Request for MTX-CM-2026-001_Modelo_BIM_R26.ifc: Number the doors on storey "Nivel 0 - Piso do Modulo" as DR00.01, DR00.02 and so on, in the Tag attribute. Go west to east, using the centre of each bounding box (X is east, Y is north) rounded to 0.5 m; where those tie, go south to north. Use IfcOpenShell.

First a look at what the model holds.

```python
import ifcopenshell
import ifcopenshell.util.element
import ifcopenshell.util.placement

model = ifcopenshell.open("MTX-CM-2026-001_Modelo_BIM_R26.ifc")
print(model.schema)
storey = next(s for s in model.by_type("IfcBuildingStorey") if s.Name == "Nivel 0 - Piso do Modulo")
doors = [e for e in ifcopenshell.util.element.get_decomposition(storey) if e.is_a("IfcDoor")]
for e in sorted(doors, key=lambda e: e.id()):
    origin = ifcopenshell.util.placement.get_local_placement(e.ObjectPlacement)[:3, 3]
    print(e.id(), e.Tag, e.Name, origin.round(2) + 0.0, sep=" | ")
```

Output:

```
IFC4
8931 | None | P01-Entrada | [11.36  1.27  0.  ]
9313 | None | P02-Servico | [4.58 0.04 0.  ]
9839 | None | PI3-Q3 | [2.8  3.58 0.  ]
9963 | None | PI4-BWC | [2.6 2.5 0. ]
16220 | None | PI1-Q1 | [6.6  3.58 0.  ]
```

```python
import ifcopenshell
import ifcopenshell.geom
import ifcopenshell.util.element
import ifcopenshell.util.shape

model = ifcopenshell.open("MTX-CM-2026-001_Modelo_BIM_R26.ifc")
settings = ifcopenshell.geom.settings()
settings.set("use-world-coords", True)


def centre(element):
    shape = ifcopenshell.geom.create_shape(settings, element)
    return ifcopenshell.util.shape.get_bbox_centroid(shape.geometry)


storey = next(s for s in model.by_type("IfcBuildingStorey") if s.Name == "Nivel 0 - Piso do Modulo")
doors = [e for e in ifcopenshell.util.element.get_decomposition(storey) if e.is_a("IfcDoor")]

# Insertion points can sit at a corner or the storey origin, so sort by the geometry (in metres).
centres = {e: centre(e) for e in doors}
doors.sort(key=lambda e: (round(centres[e][0] / 0.5), centres[e][1]))

for i, e in enumerate(doors, start=1):
    number = f"DR00.{i:02d}"
    e.Tag = number
    print(e.id(), number)

model.write("MTX-CM-2026-001_Modelo_BIM_R26_rev.ifc")
```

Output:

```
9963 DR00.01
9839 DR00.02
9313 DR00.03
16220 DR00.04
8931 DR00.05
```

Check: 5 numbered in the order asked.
